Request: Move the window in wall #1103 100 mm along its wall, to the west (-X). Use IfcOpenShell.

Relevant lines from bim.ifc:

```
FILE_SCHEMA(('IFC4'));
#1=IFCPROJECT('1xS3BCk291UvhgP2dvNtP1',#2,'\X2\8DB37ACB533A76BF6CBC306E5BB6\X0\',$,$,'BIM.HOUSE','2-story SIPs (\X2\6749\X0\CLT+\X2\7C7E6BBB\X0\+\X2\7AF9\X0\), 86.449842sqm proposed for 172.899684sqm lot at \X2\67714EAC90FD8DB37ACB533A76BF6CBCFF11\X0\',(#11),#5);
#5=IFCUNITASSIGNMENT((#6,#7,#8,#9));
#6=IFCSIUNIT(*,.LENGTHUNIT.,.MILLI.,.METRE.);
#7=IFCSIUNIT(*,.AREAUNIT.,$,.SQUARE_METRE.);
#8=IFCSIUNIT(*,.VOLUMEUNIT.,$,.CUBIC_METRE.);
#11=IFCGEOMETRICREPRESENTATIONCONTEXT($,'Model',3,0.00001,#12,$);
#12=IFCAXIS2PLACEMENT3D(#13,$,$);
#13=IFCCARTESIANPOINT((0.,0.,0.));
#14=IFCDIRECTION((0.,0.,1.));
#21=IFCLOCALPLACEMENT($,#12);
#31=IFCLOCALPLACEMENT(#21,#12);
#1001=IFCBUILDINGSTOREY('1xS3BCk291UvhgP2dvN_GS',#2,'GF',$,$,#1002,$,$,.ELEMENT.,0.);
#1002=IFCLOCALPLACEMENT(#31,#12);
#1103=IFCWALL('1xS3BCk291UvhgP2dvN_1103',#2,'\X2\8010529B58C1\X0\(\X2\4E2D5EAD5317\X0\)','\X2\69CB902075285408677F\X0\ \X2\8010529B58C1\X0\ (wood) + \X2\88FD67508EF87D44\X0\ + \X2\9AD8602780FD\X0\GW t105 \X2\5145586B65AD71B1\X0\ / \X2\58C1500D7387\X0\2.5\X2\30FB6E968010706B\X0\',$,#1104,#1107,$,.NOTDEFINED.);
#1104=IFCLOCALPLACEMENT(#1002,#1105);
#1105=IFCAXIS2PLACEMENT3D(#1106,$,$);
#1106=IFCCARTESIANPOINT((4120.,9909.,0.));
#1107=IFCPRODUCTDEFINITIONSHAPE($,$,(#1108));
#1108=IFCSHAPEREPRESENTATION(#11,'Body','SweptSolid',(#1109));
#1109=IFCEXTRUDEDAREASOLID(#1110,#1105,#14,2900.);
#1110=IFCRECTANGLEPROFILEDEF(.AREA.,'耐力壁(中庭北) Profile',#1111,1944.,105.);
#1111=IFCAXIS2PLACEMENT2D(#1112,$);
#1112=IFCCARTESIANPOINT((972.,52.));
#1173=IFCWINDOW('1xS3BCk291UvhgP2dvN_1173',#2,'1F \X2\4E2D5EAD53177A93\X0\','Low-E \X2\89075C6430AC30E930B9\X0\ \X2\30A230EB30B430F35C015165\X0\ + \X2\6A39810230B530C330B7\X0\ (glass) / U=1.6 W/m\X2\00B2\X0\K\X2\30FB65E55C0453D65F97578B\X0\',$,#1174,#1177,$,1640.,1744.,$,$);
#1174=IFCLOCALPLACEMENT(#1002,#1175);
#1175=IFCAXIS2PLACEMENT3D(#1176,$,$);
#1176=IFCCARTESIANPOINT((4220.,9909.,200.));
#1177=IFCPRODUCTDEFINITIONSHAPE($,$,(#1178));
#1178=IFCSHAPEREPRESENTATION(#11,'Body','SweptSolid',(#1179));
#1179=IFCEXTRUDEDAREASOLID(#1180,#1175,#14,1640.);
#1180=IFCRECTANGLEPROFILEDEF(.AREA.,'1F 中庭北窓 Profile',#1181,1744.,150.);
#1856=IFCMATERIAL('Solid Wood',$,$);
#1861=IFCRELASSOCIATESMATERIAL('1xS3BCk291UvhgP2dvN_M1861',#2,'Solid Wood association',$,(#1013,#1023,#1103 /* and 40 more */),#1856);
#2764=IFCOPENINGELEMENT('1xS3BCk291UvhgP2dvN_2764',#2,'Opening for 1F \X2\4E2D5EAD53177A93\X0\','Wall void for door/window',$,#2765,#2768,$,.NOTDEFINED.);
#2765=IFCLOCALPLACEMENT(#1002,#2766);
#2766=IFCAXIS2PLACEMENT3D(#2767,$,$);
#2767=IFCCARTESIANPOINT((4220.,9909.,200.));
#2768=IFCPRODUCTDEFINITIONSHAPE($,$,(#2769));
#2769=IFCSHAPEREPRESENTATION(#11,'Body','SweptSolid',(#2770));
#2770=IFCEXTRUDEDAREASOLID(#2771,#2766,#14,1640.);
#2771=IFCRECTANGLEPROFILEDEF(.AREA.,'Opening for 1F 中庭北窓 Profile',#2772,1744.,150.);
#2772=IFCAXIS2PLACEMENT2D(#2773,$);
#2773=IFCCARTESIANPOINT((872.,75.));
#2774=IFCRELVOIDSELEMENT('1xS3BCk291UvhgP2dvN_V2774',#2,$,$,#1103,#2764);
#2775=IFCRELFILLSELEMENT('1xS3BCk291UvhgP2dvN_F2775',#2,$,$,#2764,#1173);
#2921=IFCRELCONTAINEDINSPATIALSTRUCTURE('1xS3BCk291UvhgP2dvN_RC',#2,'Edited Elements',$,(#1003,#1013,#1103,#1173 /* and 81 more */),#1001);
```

```python
import ifcopenshell
import ifcopenshell.api.geometry
import ifcopenshell.util.placement

model = ifcopenshell.open("bim.ifc")

window = model.by_guid("1xS3BCk291UvhgP2dvN_1173")
opening = window.FillsVoids[0].RelatingOpeningElement
wall = opening.VoidsElements[0].RelatingBuildingElement

wall_matrix = ifcopenshell.util.placement.get_local_placement(wall.ObjectPlacement)
shift = wall_matrix[:3, 0] * -100.0
before = ifcopenshell.util.placement.get_local_placement(window.ObjectPlacement)[:3, 3].copy()

# The window is not placed relative to its opening, so move both.
for product in (opening, window):
    matrix = ifcopenshell.util.placement.get_local_placement(product.ObjectPlacement)
    matrix[:3, 3] += shift
    ifcopenshell.api.geometry.edit_object_placement(model, product=product, matrix=matrix, is_si=False)

after = ifcopenshell.util.placement.get_local_placement(window.ObjectPlacement)[:3, 3]
print("window moved by", (after - before).round(3) + 0.0)

model.write("bim_updated.ifc")
```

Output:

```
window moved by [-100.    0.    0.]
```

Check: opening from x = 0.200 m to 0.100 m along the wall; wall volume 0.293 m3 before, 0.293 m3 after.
